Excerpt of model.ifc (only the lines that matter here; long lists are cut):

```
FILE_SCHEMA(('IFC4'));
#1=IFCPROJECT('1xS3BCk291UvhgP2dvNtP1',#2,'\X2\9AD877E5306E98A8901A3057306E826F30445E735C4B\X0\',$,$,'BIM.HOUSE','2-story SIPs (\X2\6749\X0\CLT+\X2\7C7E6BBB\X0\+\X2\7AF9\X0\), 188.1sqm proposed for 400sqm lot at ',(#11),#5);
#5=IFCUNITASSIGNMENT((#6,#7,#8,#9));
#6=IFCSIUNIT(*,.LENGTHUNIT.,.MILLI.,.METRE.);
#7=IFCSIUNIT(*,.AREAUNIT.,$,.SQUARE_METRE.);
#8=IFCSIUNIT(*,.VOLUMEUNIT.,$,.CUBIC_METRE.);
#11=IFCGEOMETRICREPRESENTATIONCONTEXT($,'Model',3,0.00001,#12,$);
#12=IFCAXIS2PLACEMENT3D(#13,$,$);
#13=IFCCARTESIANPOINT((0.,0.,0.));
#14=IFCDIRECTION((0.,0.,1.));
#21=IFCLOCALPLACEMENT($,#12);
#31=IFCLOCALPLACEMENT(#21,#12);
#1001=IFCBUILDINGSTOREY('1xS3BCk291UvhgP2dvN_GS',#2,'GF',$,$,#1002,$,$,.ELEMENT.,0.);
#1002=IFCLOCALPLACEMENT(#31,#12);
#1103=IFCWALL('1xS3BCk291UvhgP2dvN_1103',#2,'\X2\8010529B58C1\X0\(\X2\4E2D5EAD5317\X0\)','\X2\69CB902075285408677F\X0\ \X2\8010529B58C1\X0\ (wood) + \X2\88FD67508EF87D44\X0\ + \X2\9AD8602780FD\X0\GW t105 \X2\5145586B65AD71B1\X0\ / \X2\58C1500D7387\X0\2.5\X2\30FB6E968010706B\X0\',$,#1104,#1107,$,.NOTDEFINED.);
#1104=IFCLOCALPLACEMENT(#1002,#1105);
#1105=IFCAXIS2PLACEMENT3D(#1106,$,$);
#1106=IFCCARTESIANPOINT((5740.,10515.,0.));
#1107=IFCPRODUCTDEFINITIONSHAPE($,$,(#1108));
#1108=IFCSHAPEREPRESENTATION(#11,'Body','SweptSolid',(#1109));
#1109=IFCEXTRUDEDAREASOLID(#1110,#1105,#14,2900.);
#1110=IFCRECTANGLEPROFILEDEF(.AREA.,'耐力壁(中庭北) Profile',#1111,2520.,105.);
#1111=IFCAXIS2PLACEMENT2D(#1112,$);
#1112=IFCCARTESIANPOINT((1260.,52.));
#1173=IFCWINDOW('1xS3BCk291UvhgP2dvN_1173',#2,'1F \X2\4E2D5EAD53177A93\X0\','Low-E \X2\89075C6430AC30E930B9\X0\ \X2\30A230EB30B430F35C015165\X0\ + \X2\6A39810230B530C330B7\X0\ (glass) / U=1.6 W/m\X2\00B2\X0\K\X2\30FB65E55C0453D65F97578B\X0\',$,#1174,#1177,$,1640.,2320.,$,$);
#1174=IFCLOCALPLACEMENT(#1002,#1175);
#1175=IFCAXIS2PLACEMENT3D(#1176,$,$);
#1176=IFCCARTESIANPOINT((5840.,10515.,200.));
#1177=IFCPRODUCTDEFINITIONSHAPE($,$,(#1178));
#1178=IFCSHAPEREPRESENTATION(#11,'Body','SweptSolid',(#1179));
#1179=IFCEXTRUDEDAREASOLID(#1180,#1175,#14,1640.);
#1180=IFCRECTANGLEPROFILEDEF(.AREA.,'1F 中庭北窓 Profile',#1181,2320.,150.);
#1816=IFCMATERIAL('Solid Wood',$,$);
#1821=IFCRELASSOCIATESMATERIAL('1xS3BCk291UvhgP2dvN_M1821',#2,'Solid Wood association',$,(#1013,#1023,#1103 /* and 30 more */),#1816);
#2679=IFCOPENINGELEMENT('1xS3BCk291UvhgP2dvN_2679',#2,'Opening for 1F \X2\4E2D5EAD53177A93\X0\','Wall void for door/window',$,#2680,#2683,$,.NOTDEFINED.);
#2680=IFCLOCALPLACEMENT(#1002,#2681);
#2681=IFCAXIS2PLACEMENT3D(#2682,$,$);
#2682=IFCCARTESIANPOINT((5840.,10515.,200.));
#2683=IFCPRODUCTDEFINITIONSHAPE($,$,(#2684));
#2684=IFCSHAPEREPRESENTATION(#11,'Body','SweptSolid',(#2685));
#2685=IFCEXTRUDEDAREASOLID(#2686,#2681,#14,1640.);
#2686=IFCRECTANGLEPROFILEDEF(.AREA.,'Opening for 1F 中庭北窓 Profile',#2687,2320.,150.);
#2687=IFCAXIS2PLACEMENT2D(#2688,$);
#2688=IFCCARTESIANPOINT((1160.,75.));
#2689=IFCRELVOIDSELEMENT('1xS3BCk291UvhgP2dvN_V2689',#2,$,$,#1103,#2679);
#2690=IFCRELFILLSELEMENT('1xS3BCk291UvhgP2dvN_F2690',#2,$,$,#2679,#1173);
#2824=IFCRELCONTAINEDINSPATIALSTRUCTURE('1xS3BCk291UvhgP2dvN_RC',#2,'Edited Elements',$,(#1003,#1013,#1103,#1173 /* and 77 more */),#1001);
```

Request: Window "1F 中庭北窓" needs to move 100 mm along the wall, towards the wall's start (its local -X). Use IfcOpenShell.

```python
import ifcopenshell
import ifcopenshell.api.geometry
import ifcopenshell.util.placement

model = ifcopenshell.open("model.ifc")

window = model.by_guid("1xS3BCk291UvhgP2dvN_1173")
opening = window.FillsVoids[0].RelatingOpeningElement
wall = opening.VoidsElements[0].RelatingBuildingElement

wall_matrix = ifcopenshell.util.placement.get_local_placement(wall.ObjectPlacement)
shift = wall_matrix[:3, 0] * -100.0
before = ifcopenshell.util.placement.get_local_placement(window.ObjectPlacement)[:3, 3].copy()

# The window is not placed relative to its opening, so move both.
for product in (opening, window):
    matrix = ifcopenshell.util.placement.get_local_placement(product.ObjectPlacement)
    matrix[:3, 3] += shift
    ifcopenshell.api.geometry.edit_object_placement(model, product=product, matrix=matrix, is_si=False)

after = ifcopenshell.util.placement.get_local_placement(window.ObjectPlacement)[:3, 3]
print("window moved by", (after - before).round(3) + 0.0)

model.write("model_updated.ifc")
```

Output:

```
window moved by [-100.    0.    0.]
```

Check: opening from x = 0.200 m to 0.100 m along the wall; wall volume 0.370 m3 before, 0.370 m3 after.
